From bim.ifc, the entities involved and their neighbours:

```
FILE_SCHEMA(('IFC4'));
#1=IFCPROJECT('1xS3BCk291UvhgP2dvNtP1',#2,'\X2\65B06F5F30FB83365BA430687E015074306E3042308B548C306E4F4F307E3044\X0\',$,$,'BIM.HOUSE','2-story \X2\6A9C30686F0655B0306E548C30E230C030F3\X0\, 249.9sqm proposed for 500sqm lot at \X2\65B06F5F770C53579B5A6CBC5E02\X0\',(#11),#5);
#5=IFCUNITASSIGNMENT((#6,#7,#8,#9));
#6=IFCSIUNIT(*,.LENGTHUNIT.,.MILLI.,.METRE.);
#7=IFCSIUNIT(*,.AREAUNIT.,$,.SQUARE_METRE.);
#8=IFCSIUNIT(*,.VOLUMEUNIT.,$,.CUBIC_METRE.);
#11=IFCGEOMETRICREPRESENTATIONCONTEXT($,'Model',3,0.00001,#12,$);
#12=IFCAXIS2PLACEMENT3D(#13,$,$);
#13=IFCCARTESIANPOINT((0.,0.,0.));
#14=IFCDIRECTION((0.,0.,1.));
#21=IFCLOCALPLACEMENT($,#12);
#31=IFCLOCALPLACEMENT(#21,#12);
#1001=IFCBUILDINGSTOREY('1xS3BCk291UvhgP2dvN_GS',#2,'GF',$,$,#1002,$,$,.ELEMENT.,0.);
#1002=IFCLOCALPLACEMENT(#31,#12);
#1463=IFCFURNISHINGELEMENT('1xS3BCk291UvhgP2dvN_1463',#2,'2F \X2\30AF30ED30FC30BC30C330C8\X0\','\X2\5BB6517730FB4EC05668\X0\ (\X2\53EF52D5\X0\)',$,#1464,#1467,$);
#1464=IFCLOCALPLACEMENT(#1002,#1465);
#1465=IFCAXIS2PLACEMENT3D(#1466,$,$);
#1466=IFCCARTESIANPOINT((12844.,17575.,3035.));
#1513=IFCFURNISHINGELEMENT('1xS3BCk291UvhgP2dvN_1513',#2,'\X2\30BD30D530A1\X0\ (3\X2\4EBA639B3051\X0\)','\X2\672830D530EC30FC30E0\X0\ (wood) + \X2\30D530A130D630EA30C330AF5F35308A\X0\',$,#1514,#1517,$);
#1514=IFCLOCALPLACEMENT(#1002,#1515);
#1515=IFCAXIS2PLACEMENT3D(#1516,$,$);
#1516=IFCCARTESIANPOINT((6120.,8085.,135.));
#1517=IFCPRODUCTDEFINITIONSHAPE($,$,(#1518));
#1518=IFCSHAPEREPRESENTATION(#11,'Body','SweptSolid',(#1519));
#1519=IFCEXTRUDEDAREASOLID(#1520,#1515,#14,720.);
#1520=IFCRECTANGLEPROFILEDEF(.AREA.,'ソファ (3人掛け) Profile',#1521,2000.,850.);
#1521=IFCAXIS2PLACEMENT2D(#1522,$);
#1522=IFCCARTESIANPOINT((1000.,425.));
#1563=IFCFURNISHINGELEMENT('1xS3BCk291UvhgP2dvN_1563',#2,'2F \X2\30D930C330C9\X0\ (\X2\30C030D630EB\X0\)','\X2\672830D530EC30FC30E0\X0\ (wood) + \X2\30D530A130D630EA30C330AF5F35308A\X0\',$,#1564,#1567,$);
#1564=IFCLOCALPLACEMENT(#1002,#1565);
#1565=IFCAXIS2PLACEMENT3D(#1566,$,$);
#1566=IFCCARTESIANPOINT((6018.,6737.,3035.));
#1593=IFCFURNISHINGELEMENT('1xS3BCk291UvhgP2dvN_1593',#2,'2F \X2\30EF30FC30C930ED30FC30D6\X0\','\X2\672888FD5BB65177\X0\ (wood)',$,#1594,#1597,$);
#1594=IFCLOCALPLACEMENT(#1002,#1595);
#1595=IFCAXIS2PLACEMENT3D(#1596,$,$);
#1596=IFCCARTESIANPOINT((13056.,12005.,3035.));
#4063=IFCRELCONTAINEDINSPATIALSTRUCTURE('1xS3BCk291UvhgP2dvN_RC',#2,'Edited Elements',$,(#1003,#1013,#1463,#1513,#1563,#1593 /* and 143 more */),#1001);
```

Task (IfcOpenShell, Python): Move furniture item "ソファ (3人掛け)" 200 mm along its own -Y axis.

```python
import ifcopenshell
import ifcopenshell.api.geometry
import ifcopenshell.util.placement

model = ifcopenshell.open("bim.ifc")

item = model.by_guid("1xS3BCk291UvhgP2dvN_1513")
matrix = ifcopenshell.util.placement.get_local_placement(item.ObjectPlacement)
matrix[:3, 3] -= matrix[:3, 1] * 200.0
ifcopenshell.api.geometry.edit_object_placement(model, product=item, matrix=matrix, is_si=False)

print(ifcopenshell.util.placement.get_local_placement(item.ObjectPlacement).round(3) + 0.0)

model.write("bim_updated.ifc")
```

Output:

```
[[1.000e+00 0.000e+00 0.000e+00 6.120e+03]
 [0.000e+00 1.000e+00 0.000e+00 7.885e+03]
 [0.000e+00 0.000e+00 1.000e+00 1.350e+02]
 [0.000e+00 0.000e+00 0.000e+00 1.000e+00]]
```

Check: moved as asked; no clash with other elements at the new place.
